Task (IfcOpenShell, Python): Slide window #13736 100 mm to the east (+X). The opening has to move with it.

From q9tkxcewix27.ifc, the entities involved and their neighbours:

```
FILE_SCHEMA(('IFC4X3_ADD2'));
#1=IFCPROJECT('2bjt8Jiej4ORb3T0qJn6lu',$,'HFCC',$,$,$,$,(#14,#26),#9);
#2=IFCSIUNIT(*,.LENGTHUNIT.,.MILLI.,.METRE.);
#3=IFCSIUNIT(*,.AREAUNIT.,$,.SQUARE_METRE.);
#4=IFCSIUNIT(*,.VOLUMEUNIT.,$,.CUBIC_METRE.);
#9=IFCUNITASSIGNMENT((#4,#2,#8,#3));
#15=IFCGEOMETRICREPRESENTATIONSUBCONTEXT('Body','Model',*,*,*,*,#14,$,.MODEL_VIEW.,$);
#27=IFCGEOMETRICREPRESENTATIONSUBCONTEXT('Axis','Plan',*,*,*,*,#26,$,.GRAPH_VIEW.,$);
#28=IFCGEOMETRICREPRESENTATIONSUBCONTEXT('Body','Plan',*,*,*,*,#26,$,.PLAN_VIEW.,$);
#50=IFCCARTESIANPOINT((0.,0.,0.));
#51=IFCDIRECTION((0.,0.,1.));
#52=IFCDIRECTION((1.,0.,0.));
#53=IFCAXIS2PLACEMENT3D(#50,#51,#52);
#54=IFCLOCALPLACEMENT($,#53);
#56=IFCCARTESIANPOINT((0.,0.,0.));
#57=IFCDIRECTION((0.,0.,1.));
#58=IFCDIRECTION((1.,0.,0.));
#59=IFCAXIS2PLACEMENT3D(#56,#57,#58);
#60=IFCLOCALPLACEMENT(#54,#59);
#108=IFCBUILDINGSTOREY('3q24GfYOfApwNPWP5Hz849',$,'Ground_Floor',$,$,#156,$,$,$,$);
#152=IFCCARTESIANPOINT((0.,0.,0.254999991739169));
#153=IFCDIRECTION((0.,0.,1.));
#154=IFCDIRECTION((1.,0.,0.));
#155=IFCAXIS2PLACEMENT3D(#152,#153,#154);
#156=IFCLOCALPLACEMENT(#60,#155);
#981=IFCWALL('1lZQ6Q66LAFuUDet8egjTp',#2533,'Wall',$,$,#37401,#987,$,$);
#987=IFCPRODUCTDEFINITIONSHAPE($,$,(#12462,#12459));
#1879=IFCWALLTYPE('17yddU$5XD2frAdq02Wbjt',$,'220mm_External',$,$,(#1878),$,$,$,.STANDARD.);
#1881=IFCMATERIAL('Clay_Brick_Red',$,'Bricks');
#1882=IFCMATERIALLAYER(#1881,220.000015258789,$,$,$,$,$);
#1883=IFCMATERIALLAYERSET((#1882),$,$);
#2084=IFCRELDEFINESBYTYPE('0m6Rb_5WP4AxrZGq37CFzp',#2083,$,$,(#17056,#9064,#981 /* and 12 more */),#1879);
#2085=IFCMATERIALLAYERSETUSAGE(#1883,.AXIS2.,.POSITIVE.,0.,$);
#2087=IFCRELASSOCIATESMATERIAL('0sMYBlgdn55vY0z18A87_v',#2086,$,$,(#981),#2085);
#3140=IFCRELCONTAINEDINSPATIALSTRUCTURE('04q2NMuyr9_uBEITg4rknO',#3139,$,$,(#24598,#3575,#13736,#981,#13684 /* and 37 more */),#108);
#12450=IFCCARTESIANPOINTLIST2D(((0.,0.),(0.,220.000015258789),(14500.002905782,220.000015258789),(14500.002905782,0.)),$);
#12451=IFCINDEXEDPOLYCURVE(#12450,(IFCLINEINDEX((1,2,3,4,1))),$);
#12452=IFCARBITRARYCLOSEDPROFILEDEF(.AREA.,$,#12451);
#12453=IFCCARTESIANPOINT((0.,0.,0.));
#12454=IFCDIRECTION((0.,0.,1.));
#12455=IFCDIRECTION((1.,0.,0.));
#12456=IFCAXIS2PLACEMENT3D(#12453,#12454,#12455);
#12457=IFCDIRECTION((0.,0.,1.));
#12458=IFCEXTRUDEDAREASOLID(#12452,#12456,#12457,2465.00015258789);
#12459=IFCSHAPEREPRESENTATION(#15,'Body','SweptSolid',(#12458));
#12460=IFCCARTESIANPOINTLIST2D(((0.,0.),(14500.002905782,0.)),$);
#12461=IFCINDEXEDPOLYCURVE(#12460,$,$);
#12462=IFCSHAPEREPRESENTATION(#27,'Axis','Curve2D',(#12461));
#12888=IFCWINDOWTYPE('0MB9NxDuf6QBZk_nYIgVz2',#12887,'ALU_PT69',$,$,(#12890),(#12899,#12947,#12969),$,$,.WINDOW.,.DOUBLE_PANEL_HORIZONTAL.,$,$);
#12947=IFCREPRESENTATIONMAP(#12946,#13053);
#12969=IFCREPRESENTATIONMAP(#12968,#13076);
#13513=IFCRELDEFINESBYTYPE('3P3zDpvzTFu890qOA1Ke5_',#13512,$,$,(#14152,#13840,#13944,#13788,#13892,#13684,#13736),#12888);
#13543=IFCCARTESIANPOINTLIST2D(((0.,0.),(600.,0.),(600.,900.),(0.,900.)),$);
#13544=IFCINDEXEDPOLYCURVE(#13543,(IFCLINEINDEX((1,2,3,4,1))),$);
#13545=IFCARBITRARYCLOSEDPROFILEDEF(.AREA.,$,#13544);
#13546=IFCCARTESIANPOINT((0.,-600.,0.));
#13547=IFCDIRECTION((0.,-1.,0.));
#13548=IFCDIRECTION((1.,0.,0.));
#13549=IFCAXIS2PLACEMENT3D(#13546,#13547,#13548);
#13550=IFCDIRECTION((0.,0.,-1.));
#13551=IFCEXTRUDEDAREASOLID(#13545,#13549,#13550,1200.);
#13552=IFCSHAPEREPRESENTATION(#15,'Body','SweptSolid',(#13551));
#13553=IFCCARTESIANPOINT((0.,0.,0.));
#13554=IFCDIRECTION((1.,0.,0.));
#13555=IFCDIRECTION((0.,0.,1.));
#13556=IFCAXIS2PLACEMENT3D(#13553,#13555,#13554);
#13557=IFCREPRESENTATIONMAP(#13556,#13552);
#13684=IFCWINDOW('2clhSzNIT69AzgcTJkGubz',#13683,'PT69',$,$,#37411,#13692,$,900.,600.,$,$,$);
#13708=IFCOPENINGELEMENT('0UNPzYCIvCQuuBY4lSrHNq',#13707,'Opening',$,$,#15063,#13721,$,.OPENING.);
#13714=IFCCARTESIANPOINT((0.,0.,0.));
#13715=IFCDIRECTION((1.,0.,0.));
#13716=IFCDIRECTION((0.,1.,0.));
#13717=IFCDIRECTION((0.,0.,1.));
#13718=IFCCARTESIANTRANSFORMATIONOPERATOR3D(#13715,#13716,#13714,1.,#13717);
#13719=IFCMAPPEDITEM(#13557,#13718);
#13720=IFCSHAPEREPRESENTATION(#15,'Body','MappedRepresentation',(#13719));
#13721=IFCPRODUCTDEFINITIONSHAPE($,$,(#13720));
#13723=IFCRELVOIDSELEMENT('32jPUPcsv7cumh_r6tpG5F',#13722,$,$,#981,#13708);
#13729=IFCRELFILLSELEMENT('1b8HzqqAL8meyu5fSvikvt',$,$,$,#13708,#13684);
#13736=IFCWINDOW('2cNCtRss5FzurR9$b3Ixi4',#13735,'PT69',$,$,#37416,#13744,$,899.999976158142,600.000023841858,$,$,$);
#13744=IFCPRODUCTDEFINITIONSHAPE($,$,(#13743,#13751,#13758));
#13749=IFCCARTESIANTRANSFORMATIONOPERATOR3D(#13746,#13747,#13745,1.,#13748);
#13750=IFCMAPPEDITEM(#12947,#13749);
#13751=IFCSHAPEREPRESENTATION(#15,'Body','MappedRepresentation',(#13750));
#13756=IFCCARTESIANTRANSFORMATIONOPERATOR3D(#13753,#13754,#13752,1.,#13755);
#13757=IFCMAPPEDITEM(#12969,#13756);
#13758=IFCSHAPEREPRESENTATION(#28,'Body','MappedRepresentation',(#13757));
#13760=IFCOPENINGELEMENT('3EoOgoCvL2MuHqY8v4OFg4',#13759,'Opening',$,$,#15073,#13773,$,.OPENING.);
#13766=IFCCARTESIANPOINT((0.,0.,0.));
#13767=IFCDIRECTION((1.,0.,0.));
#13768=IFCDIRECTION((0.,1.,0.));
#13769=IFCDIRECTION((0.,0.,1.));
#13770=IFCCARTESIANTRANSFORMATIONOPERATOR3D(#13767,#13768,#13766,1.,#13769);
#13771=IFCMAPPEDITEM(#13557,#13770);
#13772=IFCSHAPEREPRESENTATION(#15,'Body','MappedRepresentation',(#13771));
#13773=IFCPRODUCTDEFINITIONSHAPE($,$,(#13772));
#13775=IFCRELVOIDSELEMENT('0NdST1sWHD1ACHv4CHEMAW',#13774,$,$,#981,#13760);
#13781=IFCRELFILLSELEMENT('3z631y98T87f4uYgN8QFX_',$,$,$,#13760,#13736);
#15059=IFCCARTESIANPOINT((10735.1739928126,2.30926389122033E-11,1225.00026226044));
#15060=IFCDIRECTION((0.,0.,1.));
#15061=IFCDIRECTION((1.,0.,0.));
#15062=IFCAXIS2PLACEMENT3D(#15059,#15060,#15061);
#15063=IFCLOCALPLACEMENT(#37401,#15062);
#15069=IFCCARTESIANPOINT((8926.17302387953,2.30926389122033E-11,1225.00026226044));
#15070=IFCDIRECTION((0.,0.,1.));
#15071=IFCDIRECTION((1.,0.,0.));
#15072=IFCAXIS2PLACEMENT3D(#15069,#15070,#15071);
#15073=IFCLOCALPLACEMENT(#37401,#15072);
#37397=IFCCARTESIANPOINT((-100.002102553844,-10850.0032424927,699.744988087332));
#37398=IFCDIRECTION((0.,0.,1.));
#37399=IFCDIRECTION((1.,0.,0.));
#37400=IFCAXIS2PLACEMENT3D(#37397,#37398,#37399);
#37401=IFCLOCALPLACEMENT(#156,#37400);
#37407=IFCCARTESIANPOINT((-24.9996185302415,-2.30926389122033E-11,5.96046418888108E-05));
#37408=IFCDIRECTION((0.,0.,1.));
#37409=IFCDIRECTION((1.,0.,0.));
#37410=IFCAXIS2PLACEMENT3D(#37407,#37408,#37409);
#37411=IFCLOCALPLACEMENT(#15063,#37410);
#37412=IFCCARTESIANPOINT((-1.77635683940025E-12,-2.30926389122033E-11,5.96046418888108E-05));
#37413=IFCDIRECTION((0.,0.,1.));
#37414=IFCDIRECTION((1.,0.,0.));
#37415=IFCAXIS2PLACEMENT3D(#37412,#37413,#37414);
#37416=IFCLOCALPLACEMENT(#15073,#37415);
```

```python
import ifcopenshell
import ifcopenshell.api.geometry
import ifcopenshell.util.placement

model = ifcopenshell.open("q9tkxcewix27.ifc")

window = model.by_guid("2cNCtRss5FzurR9$b3Ixi4")
opening = window.FillsVoids[0].RelatingOpeningElement
wall = opening.VoidsElements[0].RelatingBuildingElement

wall_matrix = ifcopenshell.util.placement.get_local_placement(wall.ObjectPlacement)
shift = wall_matrix[:3, 0] * 100.0
before = ifcopenshell.util.placement.get_local_placement(window.ObjectPlacement)[:3, 3].copy()

# The window is placed relative to its opening, so it follows when the opening moves.
matrix = ifcopenshell.util.placement.get_local_placement(opening.ObjectPlacement)
matrix[:3, 3] += shift
ifcopenshell.api.geometry.edit_object_placement(
    model, product=opening, matrix=matrix, is_si=False, should_transform_children=True
)

after = ifcopenshell.util.placement.get_local_placement(window.ObjectPlacement)[:3, 3]
print("window moved by", (after - before).round(3) + 0.0)

model.write("q9tkxcewix27_updated.ifc")
```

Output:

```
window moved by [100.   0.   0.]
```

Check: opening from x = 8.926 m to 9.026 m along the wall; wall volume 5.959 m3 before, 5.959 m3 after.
